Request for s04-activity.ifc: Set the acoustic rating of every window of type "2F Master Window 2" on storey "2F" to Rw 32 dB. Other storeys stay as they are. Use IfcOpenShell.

First a look at what the model holds.

```python
import ifcopenshell
import ifcopenshell.util.element

model = ifcopenshell.open("s04-activity.ifc")
print(model.schema)
storey = next(s for s in model.by_type("IfcBuildingStorey") if s.Name == "2F")
windows = [e for e in ifcopenshell.util.element.get_decomposition(storey) if e.is_a("IfcWindow")]
seen = {}
for e in windows:
    element_type = ifcopenshell.util.element.get_type(e)
    key = (element_type.Name if element_type != e and element_type else None, ifcopenshell.util.element.get_pset(e, "Pset_WindowCommon", "AcousticRating"))
    seen[key] = seen.get(key, 0) + 1
for (name, value), count in sorted(seen.items(), key=str):
    print(count, "x", name, "|", value)
```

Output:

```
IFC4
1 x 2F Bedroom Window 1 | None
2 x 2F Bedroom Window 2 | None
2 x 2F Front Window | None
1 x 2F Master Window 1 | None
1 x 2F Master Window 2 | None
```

```python
import ifcopenshell
import ifcopenshell.api.pset
import ifcopenshell.util.element

model = ifcopenshell.open("s04-activity.ifc")

storey = next(s for s in model.by_type("IfcBuildingStorey") if s.Name == "2F")
windows = [e for e in ifcopenshell.util.element.get_decomposition(storey) if e.is_a("IfcWindow")]

count = 0
for e in windows:
    element_type = ifcopenshell.util.element.get_type(e)
    if element_type in (None, e) or element_type.Name != "2F Master Window 2":
        continue
    # add_pset returns the element's existing set when there is one.
    pset = ifcopenshell.api.pset.add_pset(model, product=e, name="Pset_WindowCommon")
    ifcopenshell.api.pset.edit_pset(model, pset=pset, properties={"AcousticRating": "Rw 32 dB"})
    count += 1

print(count, "windows updated")

model.write("s04-activity_v2.ifc")
```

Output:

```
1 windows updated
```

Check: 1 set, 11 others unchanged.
